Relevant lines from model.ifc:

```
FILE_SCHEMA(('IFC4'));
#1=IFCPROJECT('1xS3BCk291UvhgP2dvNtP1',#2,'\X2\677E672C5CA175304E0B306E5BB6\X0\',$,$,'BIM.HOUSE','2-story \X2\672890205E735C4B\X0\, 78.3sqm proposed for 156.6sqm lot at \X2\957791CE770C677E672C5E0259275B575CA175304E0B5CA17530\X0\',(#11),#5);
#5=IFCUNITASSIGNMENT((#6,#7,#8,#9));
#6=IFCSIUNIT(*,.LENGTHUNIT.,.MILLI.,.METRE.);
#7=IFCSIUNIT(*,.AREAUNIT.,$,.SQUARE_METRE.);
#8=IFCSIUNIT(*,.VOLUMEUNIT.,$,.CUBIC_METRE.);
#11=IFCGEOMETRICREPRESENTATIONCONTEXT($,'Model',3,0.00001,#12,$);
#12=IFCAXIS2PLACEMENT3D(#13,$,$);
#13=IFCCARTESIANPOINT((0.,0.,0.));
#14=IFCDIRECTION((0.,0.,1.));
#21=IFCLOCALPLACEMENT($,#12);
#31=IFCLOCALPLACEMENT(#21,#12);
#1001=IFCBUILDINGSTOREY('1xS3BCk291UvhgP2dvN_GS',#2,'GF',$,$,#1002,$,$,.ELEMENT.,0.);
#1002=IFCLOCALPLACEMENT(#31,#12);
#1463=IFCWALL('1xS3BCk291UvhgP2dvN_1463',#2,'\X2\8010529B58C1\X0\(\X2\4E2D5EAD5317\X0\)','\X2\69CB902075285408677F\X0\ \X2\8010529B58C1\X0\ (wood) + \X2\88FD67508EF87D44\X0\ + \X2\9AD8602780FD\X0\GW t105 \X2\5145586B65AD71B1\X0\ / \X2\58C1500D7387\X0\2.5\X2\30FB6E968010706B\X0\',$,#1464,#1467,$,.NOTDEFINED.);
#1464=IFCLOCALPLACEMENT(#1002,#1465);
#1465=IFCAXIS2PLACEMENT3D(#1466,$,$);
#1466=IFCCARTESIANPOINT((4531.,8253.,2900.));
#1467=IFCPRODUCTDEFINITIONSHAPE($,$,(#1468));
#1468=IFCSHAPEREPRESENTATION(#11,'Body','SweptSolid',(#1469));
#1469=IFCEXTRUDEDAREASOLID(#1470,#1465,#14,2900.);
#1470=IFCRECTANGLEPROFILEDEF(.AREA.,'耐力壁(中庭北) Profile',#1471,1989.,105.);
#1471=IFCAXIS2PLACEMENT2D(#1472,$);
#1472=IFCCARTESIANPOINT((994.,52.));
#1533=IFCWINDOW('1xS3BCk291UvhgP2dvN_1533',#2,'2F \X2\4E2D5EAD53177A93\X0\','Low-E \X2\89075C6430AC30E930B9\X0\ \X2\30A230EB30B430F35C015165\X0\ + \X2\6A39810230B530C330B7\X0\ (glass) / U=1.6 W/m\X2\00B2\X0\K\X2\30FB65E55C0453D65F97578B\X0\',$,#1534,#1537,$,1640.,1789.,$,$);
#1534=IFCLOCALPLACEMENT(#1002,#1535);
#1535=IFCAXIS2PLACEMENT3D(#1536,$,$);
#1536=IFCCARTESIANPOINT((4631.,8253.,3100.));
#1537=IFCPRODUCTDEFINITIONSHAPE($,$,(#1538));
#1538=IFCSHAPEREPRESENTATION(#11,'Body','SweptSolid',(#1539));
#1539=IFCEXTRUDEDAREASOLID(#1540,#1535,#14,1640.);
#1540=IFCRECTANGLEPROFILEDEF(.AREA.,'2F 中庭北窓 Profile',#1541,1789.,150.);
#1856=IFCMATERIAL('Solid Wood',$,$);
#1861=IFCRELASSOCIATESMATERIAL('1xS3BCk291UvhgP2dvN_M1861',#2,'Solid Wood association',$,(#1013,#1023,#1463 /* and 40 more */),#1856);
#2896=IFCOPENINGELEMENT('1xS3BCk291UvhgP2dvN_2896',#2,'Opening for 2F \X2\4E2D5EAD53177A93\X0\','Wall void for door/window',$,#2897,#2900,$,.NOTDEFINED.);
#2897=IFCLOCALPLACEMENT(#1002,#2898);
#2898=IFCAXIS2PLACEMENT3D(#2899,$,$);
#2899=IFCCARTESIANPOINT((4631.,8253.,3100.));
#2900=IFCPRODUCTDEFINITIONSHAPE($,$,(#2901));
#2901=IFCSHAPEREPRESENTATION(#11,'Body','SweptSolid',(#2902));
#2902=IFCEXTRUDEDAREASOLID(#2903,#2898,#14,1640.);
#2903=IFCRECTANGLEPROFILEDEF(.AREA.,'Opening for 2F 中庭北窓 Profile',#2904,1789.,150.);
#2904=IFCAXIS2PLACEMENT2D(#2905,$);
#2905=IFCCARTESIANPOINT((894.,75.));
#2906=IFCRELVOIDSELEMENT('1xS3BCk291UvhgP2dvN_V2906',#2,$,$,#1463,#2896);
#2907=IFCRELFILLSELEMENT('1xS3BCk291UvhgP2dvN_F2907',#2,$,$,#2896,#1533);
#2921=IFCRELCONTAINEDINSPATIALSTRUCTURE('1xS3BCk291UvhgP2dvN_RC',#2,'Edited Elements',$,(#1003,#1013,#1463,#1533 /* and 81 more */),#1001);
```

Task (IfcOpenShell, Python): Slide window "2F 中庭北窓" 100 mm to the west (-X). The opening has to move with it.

```python
import ifcopenshell
import ifcopenshell.api.geometry
import ifcopenshell.util.placement
import ifcopenshell.util.unit

model = ifcopenshell.open("model.ifc")
unit_scale = ifcopenshell.util.unit.calculate_unit_scale(model)

window = model.by_guid("1xS3BCk291UvhgP2dvN_1533")
opening = window.FillsVoids[0].RelatingOpeningElement
wall = opening.VoidsElements[0].RelatingBuildingElement

wall_matrix = ifcopenshell.util.placement.get_local_placement(wall.ObjectPlacement)
shift = wall_matrix[:3, 0] * -0.1 / unit_scale
before = ifcopenshell.util.placement.get_local_placement(window.ObjectPlacement)[:3, 3].copy()

# The window is not placed relative to its opening, so move both.
for product in (opening, window):
    matrix = ifcopenshell.util.placement.get_local_placement(product.ObjectPlacement)
    matrix[:3, 3] += shift
    ifcopenshell.api.geometry.edit_object_placement(model, product=product, matrix=matrix, is_si=False)

after = ifcopenshell.util.placement.get_local_placement(window.ObjectPlacement)[:3, 3]
print("window moved by", (after - before).round(3) + 0.0)

model.write("model_rev.ifc")
```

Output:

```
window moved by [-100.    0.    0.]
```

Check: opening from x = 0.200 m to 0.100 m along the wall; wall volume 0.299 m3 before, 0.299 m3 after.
